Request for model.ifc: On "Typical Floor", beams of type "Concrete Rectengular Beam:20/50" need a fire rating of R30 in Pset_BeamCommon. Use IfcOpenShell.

First a look at what the model holds.

```python
import ifcopenshell
import ifcopenshell.util.element

model = ifcopenshell.open("model.ifc")
print(model.schema)
storey = next(s for s in model.by_type("IfcBuildingStorey") if s.Name == "Typical Floor")
beams = [e for e in ifcopenshell.util.element.get_decomposition(storey) if e.is_a("IfcBeam")]
seen = {}
for e in beams:
    element_type = ifcopenshell.util.element.get_type(e)
    key = (element_type.Name if element_type != e and element_type else None, ifcopenshell.util.element.get_pset(e, "Pset_BeamCommon", "FireRating"))
    seen[key] = seen.get(key, 0) + 1
for (name, value), count in sorted(seen.items(), key=str):
    print(count, "x", name, "|", value)
```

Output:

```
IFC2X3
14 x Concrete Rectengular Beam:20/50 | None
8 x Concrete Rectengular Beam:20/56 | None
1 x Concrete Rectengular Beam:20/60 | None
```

```python
import ifcopenshell
import ifcopenshell.api.pset
import ifcopenshell.util.element

model = ifcopenshell.open("model.ifc")

storey = next(s for s in model.by_type("IfcBuildingStorey") if s.Name == "Typical Floor")
beams = [e for e in ifcopenshell.util.element.get_decomposition(storey) if e.is_a("IfcBeam")]

count = 0
for e in beams:
    element_type = ifcopenshell.util.element.get_type(e)
    if element_type in (None, e) or element_type.Name != "Concrete Rectengular Beam:20/50":
        continue
    # add_pset returns the element's existing set when there is one.
    pset = ifcopenshell.api.pset.add_pset(model, product=e, name="Pset_BeamCommon")
    ifcopenshell.api.pset.edit_pset(model, pset=pset, properties={"FireRating": "R30"})
    count += 1

print(count, "beams updated")

model.write("model_v2.ifc")
```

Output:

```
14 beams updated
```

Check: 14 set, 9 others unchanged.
